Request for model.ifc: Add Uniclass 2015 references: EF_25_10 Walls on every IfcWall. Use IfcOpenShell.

First a look at what the model holds.

```python
import ifcopenshell

model = ifcopenshell.open("model.ifc")
print(model.schema)
print("classifications:", [c.Name for c in model.by_type("IfcClassification")])
for ifc_class in ("IfcDoor", "IfcRoof", "IfcStair", "IfcWall", "IfcWindow"):
    print(ifc_class, len(model.by_type(ifc_class)))
```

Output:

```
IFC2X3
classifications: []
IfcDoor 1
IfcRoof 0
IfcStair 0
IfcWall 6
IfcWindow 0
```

```python
import ifcopenshell
import ifcopenshell.api.classification

model = ifcopenshell.open("model.ifc")

# IFC2X3 requires Source and Edition and has no link from the project to the system.
system = model.create_entity("IfcClassification", Source="NBS", Edition="2015", Name="Uniclass 2015")

codes = {
    "IfcWall": ("EF_25_10", "Walls"),
}
for ifc_class, (code, name) in codes.items():
    products = model.by_type(ifc_class)
    ifcopenshell.api.classification.add_reference(
        model, products=products, classification=system, identification=code, name=name
    )
    print(code, len(products))

model.write("model_v2.ifc")
```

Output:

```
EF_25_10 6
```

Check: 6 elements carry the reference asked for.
